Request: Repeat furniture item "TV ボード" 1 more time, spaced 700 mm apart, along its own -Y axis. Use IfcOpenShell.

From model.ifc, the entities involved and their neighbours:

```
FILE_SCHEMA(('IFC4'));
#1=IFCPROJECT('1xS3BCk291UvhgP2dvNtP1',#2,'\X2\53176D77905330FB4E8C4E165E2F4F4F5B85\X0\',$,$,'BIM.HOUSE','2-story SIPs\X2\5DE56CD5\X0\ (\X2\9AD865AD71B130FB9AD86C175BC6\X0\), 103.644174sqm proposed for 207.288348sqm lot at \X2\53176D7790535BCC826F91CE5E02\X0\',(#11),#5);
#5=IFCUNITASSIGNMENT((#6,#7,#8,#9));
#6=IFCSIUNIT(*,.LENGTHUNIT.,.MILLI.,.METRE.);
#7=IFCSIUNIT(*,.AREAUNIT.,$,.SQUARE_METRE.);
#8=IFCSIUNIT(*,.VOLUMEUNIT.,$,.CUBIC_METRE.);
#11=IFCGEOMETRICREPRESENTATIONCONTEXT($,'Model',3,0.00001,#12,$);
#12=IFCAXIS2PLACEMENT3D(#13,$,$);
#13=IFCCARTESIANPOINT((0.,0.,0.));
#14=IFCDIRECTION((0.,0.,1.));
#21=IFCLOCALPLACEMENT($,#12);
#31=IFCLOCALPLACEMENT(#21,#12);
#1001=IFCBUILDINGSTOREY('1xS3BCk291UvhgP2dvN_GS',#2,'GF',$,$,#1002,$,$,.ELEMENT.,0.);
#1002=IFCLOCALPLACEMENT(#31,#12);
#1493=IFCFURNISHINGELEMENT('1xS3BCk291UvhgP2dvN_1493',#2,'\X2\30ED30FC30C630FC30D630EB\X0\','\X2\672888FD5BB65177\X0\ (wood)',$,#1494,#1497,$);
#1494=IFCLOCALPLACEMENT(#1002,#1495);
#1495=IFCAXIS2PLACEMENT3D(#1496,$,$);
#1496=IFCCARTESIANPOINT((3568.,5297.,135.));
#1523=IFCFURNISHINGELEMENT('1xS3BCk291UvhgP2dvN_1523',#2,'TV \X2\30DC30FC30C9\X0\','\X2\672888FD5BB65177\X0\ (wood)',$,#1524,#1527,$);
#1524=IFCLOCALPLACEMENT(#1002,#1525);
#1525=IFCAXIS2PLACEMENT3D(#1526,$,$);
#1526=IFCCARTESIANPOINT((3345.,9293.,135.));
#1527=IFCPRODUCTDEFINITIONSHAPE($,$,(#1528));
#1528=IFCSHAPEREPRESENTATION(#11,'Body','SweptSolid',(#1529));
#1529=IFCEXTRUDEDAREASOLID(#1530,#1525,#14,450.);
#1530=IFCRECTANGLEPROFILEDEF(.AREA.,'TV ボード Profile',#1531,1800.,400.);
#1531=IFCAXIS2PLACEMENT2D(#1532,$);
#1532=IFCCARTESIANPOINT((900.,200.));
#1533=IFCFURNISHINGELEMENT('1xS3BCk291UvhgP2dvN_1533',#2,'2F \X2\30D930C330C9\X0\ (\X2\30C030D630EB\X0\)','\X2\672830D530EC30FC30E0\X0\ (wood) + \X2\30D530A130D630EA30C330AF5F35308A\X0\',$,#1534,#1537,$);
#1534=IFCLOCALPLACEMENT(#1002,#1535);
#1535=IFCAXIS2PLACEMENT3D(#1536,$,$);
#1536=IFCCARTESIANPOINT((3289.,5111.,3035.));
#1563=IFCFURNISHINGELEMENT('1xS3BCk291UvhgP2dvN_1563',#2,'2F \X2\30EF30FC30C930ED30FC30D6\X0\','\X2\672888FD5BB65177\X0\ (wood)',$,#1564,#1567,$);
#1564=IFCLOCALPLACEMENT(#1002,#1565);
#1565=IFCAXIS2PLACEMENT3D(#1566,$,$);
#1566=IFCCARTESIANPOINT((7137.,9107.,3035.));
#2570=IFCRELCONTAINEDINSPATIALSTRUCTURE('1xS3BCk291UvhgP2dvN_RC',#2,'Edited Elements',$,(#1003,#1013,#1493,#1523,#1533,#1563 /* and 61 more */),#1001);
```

```python
import ifcopenshell
import ifcopenshell.api.geometry
import ifcopenshell.api.root
import ifcopenshell.util.element
import ifcopenshell.util.placement
import ifcopenshell.util.unit

model = ifcopenshell.open("model.ifc")
unit_scale = ifcopenshell.util.unit.calculate_unit_scale(model)


def reuse_history(source, copy):
    """copy_class also copies each property set's owner history, people and application; keep the originals."""
    for rel in copy.IsDefinedBy:
        if rel.is_a("IfcRelDefinesByProperties") and (history := rel.RelatingPropertyDefinition.OwnerHistory):
            rel.RelatingPropertyDefinition.OwnerHistory = source.OwnerHistory
            ifcopenshell.util.element.remove_deep2(model, history)


source = model.by_guid("1xS3BCk291UvhgP2dvN_1523")
base = ifcopenshell.util.placement.get_local_placement(source.ObjectPlacement)
step = -base[:3, 1] * 0.7 / unit_scale

for i in range(1, 2):
    copy = ifcopenshell.api.root.copy_class(model, product=source)
    copy.Representation = ifcopenshell.util.element.copy_deep(
        model, source.Representation, exclude=["IfcGeometricRepresentationContext", "IfcRepresentationMap"]
    )
    reuse_history(source, copy)
    matrix = base.copy()
    matrix[:3, 3] += i * step
    print("added at", matrix[:3, 3].round(3) + 0.0)
    ifcopenshell.api.geometry.edit_object_placement(model, product=copy, matrix=matrix, is_si=False)

model.write("model_rev.ifc")
```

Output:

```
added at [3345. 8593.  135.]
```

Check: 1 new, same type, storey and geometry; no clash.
